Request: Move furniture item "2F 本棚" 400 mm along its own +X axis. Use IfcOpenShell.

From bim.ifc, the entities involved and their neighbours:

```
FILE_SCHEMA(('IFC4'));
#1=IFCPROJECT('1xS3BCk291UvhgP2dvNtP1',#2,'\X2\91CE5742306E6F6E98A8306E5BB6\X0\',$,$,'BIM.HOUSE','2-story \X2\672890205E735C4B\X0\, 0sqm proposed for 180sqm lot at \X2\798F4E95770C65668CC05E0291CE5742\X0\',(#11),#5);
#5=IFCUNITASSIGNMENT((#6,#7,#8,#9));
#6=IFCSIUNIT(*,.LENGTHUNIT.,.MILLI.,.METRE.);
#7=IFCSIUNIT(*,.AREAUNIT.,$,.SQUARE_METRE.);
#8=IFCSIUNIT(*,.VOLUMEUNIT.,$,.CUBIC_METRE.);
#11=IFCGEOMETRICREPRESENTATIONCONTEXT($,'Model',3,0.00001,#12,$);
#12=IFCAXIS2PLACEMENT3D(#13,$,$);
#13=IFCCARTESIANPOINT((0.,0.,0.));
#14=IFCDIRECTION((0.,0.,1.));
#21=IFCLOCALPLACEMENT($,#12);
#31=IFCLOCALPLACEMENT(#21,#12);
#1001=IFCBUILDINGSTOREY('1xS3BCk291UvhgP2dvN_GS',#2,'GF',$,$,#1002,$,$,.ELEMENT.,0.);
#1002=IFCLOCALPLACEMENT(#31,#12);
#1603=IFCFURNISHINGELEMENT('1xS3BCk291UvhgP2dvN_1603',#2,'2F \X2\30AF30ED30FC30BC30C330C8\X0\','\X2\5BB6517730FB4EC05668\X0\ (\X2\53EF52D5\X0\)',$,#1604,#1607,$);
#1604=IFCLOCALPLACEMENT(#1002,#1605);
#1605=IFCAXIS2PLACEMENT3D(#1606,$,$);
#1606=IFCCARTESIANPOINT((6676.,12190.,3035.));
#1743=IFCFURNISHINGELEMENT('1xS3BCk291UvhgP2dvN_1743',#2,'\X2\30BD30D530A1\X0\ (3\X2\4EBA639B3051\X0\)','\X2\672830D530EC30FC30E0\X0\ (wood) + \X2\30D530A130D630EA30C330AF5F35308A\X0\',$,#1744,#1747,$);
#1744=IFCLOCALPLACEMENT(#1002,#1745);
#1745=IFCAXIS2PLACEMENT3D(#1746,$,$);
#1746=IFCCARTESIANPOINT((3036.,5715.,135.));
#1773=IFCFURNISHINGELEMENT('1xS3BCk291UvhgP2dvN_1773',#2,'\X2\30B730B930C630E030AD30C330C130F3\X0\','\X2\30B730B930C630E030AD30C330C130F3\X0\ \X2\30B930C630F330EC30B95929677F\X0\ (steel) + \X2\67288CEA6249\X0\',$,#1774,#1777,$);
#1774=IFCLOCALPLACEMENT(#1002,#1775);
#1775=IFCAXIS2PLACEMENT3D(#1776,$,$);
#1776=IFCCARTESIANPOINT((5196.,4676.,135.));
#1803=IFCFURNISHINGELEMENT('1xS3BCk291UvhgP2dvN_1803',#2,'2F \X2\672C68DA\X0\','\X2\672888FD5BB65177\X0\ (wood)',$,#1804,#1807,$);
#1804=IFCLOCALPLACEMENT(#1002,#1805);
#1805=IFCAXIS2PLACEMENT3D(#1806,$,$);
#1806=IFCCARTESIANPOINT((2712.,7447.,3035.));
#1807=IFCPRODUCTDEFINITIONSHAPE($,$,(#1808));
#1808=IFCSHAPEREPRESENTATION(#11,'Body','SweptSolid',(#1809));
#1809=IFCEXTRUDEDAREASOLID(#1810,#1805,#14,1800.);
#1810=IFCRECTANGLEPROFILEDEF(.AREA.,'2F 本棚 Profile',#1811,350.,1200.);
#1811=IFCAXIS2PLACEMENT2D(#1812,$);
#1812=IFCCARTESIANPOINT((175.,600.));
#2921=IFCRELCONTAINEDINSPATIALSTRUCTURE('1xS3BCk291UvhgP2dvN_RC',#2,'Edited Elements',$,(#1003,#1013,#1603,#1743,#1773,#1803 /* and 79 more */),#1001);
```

```python
import ifcopenshell
import ifcopenshell.api.geometry
import ifcopenshell.util.placement
import ifcopenshell.util.unit

model = ifcopenshell.open("bim.ifc")
unit_scale = ifcopenshell.util.unit.calculate_unit_scale(model)

item = model.by_guid("1xS3BCk291UvhgP2dvN_1803")
matrix = ifcopenshell.util.placement.get_local_placement(item.ObjectPlacement)
matrix[:3, 3] += matrix[:3, 0] * 0.4 / unit_scale
ifcopenshell.api.geometry.edit_object_placement(model, product=item, matrix=matrix, is_si=False)

print(ifcopenshell.util.placement.get_local_placement(item.ObjectPlacement).round(3) + 0.0)

model.write("bim_edited.ifc")
```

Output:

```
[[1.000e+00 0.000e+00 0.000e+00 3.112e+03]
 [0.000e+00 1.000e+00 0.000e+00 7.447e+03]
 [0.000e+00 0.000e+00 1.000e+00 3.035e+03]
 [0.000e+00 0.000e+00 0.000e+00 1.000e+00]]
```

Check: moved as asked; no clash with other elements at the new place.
